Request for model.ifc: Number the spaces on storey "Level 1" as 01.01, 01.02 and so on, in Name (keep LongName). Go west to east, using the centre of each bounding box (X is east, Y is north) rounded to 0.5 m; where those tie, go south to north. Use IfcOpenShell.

First a look at what the model holds.

```python
import ifcopenshell
import ifcopenshell.util.element
import ifcopenshell.util.placement

model = ifcopenshell.open("model.ifc")
print(model.schema)
storey = next(s for s in model.by_type("IfcBuildingStorey") if s.Name == "Level 1")
spaces = [e for e in ifcopenshell.util.element.get_decomposition(storey) if e.is_a("IfcSpace")]
for e in sorted(spaces, key=lambda e: e.id()):
    origin = ifcopenshell.util.placement.get_local_placement(e.ObjectPlacement)[:3, 3]
    print(e.id(), e.Name, e.LongName, origin.round(2) + 0.0, sep=" | ")
```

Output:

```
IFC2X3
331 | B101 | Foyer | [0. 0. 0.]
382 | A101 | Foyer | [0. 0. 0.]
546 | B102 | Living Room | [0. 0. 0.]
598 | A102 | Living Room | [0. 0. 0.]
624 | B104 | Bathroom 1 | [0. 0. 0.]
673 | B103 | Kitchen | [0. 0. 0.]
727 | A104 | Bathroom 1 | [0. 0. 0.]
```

```python
import ifcopenshell
import ifcopenshell.geom
import ifcopenshell.util.element
import ifcopenshell.util.shape

model = ifcopenshell.open("model.ifc")
settings = ifcopenshell.geom.settings()
settings.set("use-world-coords", True)


def centre(element):
    shape = ifcopenshell.geom.create_shape(settings, element)
    return ifcopenshell.util.shape.get_bbox_centroid(shape.geometry)


storey = next(s for s in model.by_type("IfcBuildingStorey") if s.Name == "Level 1")
spaces = [e for e in ifcopenshell.util.element.get_decomposition(storey) if e.is_a("IfcSpace")]

# Insertion points can sit at a corner or the storey origin, so sort by the geometry (in metres).
centres = {e: centre(e) for e in spaces}
spaces.sort(key=lambda e: (round(centres[e][0] / 0.5), centres[e][1]))

for i, e in enumerate(spaces, start=1):
    number = f"01.{i:02d}"
    e.Name = number
    print(e.id(), number)

model.write("model-out.ifc")
```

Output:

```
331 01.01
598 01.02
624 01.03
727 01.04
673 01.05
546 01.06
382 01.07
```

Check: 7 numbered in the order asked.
